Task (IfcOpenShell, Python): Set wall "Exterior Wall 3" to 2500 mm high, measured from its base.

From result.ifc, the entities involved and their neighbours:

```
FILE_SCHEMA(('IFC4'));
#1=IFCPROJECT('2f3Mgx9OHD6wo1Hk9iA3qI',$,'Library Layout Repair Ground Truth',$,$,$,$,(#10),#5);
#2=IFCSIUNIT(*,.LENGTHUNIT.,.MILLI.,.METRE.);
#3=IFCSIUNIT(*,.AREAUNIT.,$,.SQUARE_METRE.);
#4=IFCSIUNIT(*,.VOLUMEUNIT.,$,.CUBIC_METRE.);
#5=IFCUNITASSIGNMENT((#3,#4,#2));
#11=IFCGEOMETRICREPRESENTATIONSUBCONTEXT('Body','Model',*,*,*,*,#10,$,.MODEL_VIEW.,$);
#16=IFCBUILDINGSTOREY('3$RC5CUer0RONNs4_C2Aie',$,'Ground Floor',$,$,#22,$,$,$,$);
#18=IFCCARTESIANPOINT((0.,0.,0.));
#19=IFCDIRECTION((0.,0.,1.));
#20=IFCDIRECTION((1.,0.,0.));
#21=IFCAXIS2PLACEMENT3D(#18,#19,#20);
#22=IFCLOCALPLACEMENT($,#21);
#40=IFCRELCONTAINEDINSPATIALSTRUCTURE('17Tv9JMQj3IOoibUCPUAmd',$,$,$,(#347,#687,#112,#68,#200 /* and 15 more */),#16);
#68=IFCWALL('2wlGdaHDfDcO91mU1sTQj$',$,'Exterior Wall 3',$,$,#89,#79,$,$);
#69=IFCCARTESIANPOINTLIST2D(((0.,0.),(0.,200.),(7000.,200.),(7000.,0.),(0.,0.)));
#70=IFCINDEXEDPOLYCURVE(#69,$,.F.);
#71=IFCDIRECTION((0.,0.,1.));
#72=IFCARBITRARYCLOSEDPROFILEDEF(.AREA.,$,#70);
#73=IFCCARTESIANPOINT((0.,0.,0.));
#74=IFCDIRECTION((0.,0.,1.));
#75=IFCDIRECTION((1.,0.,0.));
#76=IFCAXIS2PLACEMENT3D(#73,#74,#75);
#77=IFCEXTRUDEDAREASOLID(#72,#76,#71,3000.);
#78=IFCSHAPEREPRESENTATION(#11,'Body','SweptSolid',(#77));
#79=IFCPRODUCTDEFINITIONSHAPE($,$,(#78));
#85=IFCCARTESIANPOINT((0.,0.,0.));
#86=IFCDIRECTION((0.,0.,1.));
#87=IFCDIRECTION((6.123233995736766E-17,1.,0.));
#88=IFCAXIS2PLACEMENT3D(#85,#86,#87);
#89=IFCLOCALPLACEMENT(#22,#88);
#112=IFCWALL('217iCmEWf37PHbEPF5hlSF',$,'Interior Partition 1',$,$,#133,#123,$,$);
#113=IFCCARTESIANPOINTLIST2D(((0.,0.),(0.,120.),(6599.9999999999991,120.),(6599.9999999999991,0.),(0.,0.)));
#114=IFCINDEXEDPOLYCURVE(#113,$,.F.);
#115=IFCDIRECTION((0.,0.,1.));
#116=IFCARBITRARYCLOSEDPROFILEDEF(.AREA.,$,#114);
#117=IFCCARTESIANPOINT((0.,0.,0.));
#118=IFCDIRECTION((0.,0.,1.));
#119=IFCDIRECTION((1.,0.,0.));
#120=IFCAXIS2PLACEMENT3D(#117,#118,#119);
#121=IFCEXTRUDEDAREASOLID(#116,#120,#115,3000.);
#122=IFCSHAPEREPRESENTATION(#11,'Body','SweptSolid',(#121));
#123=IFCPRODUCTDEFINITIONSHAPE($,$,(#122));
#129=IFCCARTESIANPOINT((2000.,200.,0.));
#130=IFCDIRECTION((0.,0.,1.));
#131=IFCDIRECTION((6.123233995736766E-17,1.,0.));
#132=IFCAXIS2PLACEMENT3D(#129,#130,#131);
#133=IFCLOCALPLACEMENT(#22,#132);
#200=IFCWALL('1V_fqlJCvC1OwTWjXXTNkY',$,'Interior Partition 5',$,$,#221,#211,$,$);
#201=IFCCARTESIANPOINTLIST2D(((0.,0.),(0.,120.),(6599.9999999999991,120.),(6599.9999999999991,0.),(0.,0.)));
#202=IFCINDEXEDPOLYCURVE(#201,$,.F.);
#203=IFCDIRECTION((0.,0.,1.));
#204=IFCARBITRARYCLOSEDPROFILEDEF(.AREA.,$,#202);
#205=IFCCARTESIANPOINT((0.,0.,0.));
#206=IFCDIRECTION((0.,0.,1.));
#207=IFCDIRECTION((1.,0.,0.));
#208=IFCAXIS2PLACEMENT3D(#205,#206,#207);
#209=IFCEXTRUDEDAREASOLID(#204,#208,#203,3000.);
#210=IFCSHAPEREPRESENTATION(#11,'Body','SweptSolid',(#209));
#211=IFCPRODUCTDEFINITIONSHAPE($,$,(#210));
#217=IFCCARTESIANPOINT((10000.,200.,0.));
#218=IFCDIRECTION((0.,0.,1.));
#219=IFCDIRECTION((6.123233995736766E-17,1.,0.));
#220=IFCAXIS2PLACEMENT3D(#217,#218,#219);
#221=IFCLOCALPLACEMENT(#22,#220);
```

```python
import ifcopenshell
import ifcopenshell.geom
import ifcopenshell.util.representation
import ifcopenshell.util.shape

model = ifcopenshell.open("result.ifc")
settings = ifcopenshell.geom.settings()


def volume(element):
    """Net volume in cubic metres, openings subtracted."""
    shape = ifcopenshell.geom.create_shape(settings, element)
    return ifcopenshell.util.shape.get_volume(shape.geometry)


wall = model.by_guid("2wlGdaHDfDcO91mU1sTQj$")
before = volume(wall)

body = ifcopenshell.util.representation.get_representation(wall, "Model", "Body")
solid = body.Items[0]
old_height = solid.Depth
solid.Depth = 2500.0
after = volume(wall)

print(f"height {old_height:g} -> {solid.Depth:g}, volume {before:.3f} -> {after:.3f} m3")

model.write("result_v2.ifc")
```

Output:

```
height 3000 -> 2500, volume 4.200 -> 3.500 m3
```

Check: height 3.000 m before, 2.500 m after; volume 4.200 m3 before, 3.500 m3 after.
